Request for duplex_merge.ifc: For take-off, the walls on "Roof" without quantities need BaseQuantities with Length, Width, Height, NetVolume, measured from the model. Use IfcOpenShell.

First a look at what the model holds.

```python
import ifcopenshell
import ifcopenshell.util.element
import ifcopenshell.util.unit

model = ifcopenshell.open("duplex_merge.ifc")
print(model.schema)
for unit_type in ("LENGTHUNIT", "AREAUNIT", "VOLUMEUNIT"):
    print(unit_type, ifcopenshell.util.unit.calculate_unit_scale(model, unit_type))
storey = next(s for s in model.by_type("IfcBuildingStorey") if s.Name == "Roof")
walls = [e for e in ifcopenshell.util.element.get_decomposition(storey) if e.is_a("IfcWall")]
for e in sorted(walls, key=lambda e: e.id()):
    print(e.id(), e.is_a(), e.Name, list(ifcopenshell.util.element.get_psets(e, qtos_only=True)), sep=" | ")
```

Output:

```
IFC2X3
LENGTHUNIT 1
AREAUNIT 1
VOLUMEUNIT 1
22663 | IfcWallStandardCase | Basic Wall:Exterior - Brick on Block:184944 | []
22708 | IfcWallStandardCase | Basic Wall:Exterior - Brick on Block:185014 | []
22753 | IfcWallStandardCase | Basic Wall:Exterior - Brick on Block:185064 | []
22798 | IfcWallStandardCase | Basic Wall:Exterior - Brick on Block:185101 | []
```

```python
import ifcopenshell
import ifcopenshell.api.pset
import ifcopenshell.geom
import ifcopenshell.util.element
import ifcopenshell.util.shape
import ifcopenshell.util.unit

model = ifcopenshell.open("duplex_merge.ifc")
unit_scale = ifcopenshell.util.unit.calculate_unit_scale(model)
volume_scale = ifcopenshell.util.unit.calculate_unit_scale(model, "VOLUMEUNIT")
settings = ifcopenshell.geom.settings()

storey = next(s for s in model.by_type("IfcBuildingStorey") if s.Name == "Roof")
walls = [e for e in ifcopenshell.util.element.get_decomposition(storey) if e.is_a("IfcWall")]

for e in sorted(walls, key=lambda e: e.id()):
    if ifcopenshell.util.element.get_psets(e, qtos_only=True, should_inherit=False):
        continue
    # Geometry comes back in metres, in the element's own axes.
    shape = ifcopenshell.geom.create_shape(settings, e)
    values = {
        "Length": ifcopenshell.util.shape.get_x(shape.geometry) / unit_scale,
        "Width": ifcopenshell.util.shape.get_y(shape.geometry) / unit_scale,
        "Height": ifcopenshell.util.shape.get_z(shape.geometry) / unit_scale,
        "NetVolume": ifcopenshell.util.shape.get_volume(shape.geometry) / volume_scale,
    }
    qto = ifcopenshell.api.pset.add_qto(model, product=e, name="BaseQuantities")
    ifcopenshell.api.pset.edit_qto(model, qto=qto, properties=values)
    print(e.id(), {k: round(v, 3) for k, v in values.items()})

model.write("duplex_merge_rev.ifc")
```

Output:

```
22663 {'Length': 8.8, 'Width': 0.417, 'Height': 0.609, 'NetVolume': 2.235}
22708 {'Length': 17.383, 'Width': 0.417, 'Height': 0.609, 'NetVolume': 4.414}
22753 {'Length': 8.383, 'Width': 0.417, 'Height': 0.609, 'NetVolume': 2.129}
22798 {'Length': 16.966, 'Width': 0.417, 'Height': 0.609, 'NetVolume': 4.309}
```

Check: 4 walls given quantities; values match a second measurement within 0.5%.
